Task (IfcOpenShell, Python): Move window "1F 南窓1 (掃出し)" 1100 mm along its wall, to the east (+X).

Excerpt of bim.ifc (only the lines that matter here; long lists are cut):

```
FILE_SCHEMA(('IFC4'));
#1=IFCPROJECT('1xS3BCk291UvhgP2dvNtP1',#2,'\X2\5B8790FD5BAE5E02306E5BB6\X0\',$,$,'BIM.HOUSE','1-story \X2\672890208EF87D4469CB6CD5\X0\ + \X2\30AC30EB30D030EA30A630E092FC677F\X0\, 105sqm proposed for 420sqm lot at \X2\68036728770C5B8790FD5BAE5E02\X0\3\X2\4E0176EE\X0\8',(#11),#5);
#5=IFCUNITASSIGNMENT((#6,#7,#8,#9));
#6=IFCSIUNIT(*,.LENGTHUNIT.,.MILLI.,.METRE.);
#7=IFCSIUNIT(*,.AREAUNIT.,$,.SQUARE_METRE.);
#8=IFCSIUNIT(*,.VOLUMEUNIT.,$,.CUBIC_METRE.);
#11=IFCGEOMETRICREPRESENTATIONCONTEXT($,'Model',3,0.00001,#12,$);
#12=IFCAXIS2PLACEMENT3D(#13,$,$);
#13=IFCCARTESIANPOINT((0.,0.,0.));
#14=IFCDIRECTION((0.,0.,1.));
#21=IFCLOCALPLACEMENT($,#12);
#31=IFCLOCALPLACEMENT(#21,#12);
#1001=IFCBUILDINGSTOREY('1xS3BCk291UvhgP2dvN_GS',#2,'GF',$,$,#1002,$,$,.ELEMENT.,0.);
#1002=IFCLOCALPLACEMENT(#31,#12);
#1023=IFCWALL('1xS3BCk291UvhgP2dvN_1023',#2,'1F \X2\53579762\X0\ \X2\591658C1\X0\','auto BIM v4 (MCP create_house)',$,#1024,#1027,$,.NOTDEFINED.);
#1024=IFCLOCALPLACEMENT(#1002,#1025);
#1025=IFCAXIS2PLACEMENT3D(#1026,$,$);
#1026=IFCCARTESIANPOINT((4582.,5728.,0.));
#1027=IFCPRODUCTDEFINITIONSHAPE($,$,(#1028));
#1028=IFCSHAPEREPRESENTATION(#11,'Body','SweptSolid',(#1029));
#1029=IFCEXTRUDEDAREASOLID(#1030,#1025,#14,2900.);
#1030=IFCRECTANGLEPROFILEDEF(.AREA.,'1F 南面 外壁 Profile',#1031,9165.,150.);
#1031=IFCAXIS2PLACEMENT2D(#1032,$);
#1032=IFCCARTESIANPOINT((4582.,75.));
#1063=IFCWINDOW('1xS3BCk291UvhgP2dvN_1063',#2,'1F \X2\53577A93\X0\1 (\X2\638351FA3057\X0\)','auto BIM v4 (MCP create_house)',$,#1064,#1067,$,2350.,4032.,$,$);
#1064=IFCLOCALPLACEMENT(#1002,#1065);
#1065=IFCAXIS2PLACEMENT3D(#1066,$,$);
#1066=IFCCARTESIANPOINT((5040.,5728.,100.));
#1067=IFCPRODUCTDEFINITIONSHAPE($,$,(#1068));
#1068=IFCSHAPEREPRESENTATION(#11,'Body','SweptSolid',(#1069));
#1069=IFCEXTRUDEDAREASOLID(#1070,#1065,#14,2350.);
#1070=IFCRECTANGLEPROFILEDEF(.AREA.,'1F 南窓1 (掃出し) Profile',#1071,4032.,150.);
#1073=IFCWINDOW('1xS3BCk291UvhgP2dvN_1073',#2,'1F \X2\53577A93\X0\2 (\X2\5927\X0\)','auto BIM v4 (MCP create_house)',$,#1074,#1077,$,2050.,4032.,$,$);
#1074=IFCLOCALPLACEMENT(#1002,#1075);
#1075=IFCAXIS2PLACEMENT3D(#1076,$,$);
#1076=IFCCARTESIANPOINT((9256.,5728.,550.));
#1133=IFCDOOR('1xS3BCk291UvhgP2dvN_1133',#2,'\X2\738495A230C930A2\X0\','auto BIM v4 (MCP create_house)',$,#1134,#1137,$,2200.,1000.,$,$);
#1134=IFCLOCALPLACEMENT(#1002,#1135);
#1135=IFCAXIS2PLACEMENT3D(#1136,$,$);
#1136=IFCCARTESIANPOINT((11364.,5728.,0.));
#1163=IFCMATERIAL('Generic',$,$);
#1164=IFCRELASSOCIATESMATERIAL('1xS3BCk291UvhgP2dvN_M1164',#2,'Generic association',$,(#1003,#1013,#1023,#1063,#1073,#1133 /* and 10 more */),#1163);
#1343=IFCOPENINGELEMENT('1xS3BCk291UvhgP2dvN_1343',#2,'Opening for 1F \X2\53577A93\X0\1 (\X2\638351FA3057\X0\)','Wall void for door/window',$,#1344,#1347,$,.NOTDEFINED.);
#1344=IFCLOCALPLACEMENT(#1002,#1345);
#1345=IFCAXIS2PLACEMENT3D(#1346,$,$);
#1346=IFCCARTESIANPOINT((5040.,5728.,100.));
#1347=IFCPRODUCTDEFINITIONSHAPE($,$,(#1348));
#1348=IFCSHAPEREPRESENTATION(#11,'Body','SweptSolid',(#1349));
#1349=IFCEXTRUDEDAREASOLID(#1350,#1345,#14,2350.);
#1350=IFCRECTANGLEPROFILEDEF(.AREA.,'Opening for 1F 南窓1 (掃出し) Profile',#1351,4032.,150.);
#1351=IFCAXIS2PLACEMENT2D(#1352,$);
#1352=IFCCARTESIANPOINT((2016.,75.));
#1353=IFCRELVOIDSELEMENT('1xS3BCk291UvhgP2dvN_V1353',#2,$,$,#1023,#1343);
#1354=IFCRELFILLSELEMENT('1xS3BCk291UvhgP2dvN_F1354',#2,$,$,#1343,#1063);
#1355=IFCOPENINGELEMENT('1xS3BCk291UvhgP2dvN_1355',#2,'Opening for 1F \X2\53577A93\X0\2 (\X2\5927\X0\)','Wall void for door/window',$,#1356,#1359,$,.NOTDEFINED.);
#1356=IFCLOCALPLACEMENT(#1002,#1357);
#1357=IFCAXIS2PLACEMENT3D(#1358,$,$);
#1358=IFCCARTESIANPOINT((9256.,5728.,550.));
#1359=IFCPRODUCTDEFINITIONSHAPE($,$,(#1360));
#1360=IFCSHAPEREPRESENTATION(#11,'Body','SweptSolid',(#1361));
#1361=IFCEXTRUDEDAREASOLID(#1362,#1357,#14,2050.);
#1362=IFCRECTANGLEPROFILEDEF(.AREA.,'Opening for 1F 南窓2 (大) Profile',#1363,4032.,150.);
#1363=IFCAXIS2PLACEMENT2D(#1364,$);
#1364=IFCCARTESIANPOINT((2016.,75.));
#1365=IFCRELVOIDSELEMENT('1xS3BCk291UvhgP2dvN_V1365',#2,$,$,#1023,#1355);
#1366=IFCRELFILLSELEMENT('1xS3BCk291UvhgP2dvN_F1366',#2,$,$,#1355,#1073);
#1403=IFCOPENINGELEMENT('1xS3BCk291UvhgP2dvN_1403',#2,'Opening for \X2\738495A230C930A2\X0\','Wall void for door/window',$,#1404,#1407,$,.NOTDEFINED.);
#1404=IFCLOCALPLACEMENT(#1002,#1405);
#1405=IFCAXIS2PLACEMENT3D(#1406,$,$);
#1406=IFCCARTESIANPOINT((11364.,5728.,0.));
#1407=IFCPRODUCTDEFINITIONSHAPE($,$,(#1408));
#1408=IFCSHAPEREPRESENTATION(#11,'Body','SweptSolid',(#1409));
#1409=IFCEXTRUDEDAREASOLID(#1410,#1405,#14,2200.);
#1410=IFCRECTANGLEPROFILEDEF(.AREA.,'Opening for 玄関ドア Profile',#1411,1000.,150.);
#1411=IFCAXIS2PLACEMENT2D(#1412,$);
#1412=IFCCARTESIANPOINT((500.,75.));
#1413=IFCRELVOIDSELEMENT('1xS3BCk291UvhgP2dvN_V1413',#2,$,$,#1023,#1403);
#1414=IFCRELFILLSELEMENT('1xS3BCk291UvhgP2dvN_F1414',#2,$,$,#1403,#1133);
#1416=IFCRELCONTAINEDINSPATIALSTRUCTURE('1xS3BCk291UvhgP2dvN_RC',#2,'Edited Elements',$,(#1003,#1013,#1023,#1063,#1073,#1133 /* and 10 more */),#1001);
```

```python
import ifcopenshell
import ifcopenshell.api.geometry
import ifcopenshell.util.placement
import ifcopenshell.util.unit

model = ifcopenshell.open("bim.ifc")
unit_scale = ifcopenshell.util.unit.calculate_unit_scale(model)

window = model.by_guid("1xS3BCk291UvhgP2dvN_1063")
opening = window.FillsVoids[0].RelatingOpeningElement
wall = opening.VoidsElements[0].RelatingBuildingElement

wall_matrix = ifcopenshell.util.placement.get_local_placement(wall.ObjectPlacement)
shift = wall_matrix[:3, 0] * 1.1 / unit_scale
before = ifcopenshell.util.placement.get_local_placement(window.ObjectPlacement)[:3, 3].copy()

# The window is not placed relative to its opening, so move both.
for product in (opening, window):
    matrix = ifcopenshell.util.placement.get_local_placement(product.ObjectPlacement)
    matrix[:3, 3] += shift
    ifcopenshell.api.geometry.edit_object_placement(model, product=product, matrix=matrix, is_si=False)

after = ifcopenshell.util.placement.get_local_placement(window.ObjectPlacement)[:3, 3]
print("window moved by", (after - before).round(3) + 0.0)

model.write("bim-out.ifc")
```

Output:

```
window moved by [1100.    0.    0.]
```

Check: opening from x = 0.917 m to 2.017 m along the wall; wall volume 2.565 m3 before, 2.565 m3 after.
